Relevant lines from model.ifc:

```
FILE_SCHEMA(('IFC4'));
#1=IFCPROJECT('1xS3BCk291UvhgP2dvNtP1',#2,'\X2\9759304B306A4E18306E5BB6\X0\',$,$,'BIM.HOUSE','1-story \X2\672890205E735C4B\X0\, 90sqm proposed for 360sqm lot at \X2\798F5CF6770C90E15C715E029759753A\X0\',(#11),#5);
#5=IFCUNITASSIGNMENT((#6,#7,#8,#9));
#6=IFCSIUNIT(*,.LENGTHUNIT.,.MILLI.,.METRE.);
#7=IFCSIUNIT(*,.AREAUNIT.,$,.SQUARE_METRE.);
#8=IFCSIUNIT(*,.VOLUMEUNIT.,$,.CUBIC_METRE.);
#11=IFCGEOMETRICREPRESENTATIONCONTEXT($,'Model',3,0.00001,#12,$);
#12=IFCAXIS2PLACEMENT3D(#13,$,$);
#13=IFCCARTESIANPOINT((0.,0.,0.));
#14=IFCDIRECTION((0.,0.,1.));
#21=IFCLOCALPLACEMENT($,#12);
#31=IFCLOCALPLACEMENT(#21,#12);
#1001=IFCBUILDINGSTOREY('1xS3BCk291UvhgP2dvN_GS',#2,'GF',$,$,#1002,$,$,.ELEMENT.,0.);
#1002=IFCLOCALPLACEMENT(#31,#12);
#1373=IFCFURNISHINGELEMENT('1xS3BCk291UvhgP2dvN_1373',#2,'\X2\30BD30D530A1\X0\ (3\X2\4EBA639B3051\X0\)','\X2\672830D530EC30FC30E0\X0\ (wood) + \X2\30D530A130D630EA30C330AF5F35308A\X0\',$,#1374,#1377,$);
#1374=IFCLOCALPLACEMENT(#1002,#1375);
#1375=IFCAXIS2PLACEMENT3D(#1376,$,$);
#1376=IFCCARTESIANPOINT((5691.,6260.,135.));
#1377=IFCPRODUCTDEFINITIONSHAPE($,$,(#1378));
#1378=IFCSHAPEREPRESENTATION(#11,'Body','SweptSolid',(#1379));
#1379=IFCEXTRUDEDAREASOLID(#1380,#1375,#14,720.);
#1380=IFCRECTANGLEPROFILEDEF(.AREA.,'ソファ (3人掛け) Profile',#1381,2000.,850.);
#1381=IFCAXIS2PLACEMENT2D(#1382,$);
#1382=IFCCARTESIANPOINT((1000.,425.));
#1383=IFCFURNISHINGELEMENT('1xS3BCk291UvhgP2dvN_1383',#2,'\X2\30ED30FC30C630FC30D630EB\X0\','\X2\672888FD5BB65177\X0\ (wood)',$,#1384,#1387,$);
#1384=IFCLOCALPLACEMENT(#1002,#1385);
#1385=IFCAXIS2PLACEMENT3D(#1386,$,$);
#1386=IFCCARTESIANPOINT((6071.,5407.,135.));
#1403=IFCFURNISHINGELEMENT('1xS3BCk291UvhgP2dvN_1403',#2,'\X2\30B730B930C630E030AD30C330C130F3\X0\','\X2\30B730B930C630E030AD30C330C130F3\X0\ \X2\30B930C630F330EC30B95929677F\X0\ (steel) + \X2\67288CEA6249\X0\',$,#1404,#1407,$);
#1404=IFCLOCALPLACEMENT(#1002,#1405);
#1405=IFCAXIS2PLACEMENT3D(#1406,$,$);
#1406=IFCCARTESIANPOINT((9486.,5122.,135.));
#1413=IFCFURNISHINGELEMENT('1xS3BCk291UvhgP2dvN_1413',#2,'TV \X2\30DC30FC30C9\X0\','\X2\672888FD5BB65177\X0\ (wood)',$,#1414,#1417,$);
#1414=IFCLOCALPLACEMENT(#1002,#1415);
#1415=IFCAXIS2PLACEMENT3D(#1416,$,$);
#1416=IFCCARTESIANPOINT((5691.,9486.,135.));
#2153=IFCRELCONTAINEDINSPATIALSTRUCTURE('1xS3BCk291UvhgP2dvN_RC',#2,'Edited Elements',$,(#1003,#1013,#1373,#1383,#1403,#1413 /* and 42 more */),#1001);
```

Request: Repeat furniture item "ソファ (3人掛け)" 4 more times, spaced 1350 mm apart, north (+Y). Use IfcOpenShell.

```python
import numpy as np
import ifcopenshell
import ifcopenshell.api.geometry
import ifcopenshell.api.root
import ifcopenshell.util.element
import ifcopenshell.util.placement

model = ifcopenshell.open("model.ifc")


def reuse_history(source, copy):
    """copy_class also copies each property set's owner history, people and application; keep the originals."""
    for rel in copy.IsDefinedBy:
        if rel.is_a("IfcRelDefinesByProperties") and (history := rel.RelatingPropertyDefinition.OwnerHistory):
            rel.RelatingPropertyDefinition.OwnerHistory = source.OwnerHistory
            ifcopenshell.util.element.remove_deep2(model, history)


source = model.by_guid("1xS3BCk291UvhgP2dvN_1373")
base = ifcopenshell.util.placement.get_local_placement(source.ObjectPlacement)
step = np.array([0.0, 1.0, 0.0]) * 1350.0

for i in range(1, 5):
    copy = ifcopenshell.api.root.copy_class(model, product=source)
    copy.Representation = ifcopenshell.util.element.copy_deep(
        model, source.Representation, exclude=["IfcGeometricRepresentationContext", "IfcRepresentationMap"]
    )
    reuse_history(source, copy)
    matrix = base.copy()
    matrix[:3, 3] += i * step
    print("added at", matrix[:3, 3].round(3) + 0.0)
    ifcopenshell.api.geometry.edit_object_placement(model, product=copy, matrix=matrix, is_si=False)

model.write("model_updated.ifc")
```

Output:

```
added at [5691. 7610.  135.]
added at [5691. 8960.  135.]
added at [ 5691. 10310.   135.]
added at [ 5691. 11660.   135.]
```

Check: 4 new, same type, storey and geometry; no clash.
